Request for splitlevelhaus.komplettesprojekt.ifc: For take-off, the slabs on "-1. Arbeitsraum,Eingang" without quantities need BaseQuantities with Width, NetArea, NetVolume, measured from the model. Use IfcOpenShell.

First a look at what the model holds.

```python
import ifcopenshell
import ifcopenshell.util.element
import ifcopenshell.util.unit

model = ifcopenshell.open("splitlevelhaus.komplettesprojekt.ifc")
print(model.schema)
for unit_type in ("LENGTHUNIT", "AREAUNIT", "VOLUMEUNIT"):
    print(unit_type, ifcopenshell.util.unit.calculate_unit_scale(model, unit_type))
storey = next(s for s in model.by_type("IfcBuildingStorey") if s.Name == "-1. Arbeitsraum,Eingang")
slabs = [e for e in ifcopenshell.util.element.get_decomposition(storey) if e.is_a("IfcSlab")]
for e in sorted(slabs, key=lambda e: e.id()):
    print(e.id(), e.is_a(), e.Name, list(ifcopenshell.util.element.get_psets(e, qtos_only=True)), sep=" | ")
```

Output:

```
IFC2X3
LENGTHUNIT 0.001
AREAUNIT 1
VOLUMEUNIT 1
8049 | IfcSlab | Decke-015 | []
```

```python
import ifcopenshell
import ifcopenshell.api.pset
import ifcopenshell.geom
import ifcopenshell.util.element
import ifcopenshell.util.shape
import ifcopenshell.util.unit

model = ifcopenshell.open("splitlevelhaus.komplettesprojekt.ifc")
unit_scale = ifcopenshell.util.unit.calculate_unit_scale(model)
area_scale = ifcopenshell.util.unit.calculate_unit_scale(model, "AREAUNIT")
volume_scale = ifcopenshell.util.unit.calculate_unit_scale(model, "VOLUMEUNIT")
settings = ifcopenshell.geom.settings()

storey = next(s for s in model.by_type("IfcBuildingStorey") if s.Name == "-1. Arbeitsraum,Eingang")
slabs = [e for e in ifcopenshell.util.element.get_decomposition(storey) if e.is_a("IfcSlab")]

for e in sorted(slabs, key=lambda e: e.id()):
    if ifcopenshell.util.element.get_psets(e, qtos_only=True, should_inherit=False):
        continue
    # Geometry comes back in metres, in the element's own axes.
    shape = ifcopenshell.geom.create_shape(settings, e)
    values = {
        "Width": ifcopenshell.util.shape.get_z(shape.geometry) / unit_scale,
        "NetArea": ifcopenshell.util.shape.get_footprint_area(shape.geometry) / area_scale,
        "NetVolume": ifcopenshell.util.shape.get_volume(shape.geometry) / volume_scale,
    }
    qto = ifcopenshell.api.pset.add_qto(model, product=e, name="BaseQuantities")
    ifcopenshell.api.pset.edit_qto(model, qto=qto, properties=values)
    print(e.id(), {k: round(v, 3) for k, v in values.items()})

model.write("splitlevelhaus.komplettesprojekt_updated.ifc")
```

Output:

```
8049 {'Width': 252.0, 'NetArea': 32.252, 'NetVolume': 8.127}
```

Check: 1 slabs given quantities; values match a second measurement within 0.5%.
